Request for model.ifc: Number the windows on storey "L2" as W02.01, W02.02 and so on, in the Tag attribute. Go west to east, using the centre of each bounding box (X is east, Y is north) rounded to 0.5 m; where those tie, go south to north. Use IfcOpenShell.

First a look at what the model holds.

```python
import ifcopenshell
import ifcopenshell.util.element
import ifcopenshell.util.placement

model = ifcopenshell.open("model.ifc")
print(model.schema)
storey = next(s for s in model.by_type("IfcBuildingStorey") if s.Name == "L2")
windows = [e for e in ifcopenshell.util.element.get_decomposition(storey) if e.is_a("IfcWindow")]
for e in sorted(windows, key=lambda e: e.id()):
    origin = ifcopenshell.util.placement.get_local_placement(e.ObjectPlacement)[:3, 3]
    print(e.id(), e.Tag, e.Name, origin.round(2) + 0.0, sep=" | ")
```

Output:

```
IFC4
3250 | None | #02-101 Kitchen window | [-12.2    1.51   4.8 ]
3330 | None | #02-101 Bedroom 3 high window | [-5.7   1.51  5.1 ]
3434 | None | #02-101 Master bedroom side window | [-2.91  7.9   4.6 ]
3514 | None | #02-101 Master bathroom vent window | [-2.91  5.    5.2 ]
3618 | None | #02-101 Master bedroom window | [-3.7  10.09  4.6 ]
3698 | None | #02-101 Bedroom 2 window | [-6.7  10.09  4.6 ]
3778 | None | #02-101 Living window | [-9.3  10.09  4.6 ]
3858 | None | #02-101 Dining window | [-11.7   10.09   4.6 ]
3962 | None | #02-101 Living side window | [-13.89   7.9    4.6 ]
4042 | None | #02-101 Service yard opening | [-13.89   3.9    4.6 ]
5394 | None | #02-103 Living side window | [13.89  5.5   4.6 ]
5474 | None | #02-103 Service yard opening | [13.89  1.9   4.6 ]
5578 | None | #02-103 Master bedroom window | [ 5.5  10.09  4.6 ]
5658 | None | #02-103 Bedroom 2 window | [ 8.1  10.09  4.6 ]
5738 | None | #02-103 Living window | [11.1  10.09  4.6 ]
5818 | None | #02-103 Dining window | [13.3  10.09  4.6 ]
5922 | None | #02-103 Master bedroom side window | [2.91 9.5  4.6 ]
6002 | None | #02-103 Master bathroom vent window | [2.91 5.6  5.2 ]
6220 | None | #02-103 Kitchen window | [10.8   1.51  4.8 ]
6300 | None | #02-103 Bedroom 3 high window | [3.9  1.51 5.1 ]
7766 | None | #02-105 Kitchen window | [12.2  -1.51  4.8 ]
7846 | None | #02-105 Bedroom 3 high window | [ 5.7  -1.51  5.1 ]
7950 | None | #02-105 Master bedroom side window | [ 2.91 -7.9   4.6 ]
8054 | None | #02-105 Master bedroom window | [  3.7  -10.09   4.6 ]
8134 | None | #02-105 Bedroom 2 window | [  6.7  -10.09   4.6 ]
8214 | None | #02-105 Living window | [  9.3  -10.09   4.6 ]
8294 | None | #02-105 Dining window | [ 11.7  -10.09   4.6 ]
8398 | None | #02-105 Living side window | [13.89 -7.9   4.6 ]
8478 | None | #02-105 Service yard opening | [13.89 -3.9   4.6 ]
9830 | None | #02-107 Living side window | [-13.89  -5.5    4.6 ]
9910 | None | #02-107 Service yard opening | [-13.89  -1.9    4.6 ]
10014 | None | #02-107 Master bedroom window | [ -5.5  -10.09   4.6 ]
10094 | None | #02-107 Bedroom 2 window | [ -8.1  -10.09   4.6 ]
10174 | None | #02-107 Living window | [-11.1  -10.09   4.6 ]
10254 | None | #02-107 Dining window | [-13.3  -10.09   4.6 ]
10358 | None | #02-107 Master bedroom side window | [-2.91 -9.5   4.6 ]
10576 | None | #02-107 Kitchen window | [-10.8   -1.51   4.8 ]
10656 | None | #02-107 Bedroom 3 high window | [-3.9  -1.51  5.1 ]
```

```python
import ifcopenshell
import ifcopenshell.geom
import ifcopenshell.util.element
import ifcopenshell.util.shape

model = ifcopenshell.open("model.ifc")
settings = ifcopenshell.geom.settings()
settings.set("use-world-coords", True)


def centre(element):
    shape = ifcopenshell.geom.create_shape(settings, element)
    return ifcopenshell.util.shape.get_bbox_centroid(shape.geometry)


storey = next(s for s in model.by_type("IfcBuildingStorey") if s.Name == "L2")
windows = [e for e in ifcopenshell.util.element.get_decomposition(storey) if e.is_a("IfcWindow")]

# Insertion points can sit at a corner or the storey origin, so sort by the geometry (in metres).
centres = {e: centre(e) for e in windows}
windows.sort(key=lambda e: (round(centres[e][0] / 0.5), centres[e][1]))

for i, e in enumerate(windows, start=1):
    number = f"W02.{i:02d}"
    e.Tag = number
    print(e.id(), number)

model.write("model_v2.ifc")
```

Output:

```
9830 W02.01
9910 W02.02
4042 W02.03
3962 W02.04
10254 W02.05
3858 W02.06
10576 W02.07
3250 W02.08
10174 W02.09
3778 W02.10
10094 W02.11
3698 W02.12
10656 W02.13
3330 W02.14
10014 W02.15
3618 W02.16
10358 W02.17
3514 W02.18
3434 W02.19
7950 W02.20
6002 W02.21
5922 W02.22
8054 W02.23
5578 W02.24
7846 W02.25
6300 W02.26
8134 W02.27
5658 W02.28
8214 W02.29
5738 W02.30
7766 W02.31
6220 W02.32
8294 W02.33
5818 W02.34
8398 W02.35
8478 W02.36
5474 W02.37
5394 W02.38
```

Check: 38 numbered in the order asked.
